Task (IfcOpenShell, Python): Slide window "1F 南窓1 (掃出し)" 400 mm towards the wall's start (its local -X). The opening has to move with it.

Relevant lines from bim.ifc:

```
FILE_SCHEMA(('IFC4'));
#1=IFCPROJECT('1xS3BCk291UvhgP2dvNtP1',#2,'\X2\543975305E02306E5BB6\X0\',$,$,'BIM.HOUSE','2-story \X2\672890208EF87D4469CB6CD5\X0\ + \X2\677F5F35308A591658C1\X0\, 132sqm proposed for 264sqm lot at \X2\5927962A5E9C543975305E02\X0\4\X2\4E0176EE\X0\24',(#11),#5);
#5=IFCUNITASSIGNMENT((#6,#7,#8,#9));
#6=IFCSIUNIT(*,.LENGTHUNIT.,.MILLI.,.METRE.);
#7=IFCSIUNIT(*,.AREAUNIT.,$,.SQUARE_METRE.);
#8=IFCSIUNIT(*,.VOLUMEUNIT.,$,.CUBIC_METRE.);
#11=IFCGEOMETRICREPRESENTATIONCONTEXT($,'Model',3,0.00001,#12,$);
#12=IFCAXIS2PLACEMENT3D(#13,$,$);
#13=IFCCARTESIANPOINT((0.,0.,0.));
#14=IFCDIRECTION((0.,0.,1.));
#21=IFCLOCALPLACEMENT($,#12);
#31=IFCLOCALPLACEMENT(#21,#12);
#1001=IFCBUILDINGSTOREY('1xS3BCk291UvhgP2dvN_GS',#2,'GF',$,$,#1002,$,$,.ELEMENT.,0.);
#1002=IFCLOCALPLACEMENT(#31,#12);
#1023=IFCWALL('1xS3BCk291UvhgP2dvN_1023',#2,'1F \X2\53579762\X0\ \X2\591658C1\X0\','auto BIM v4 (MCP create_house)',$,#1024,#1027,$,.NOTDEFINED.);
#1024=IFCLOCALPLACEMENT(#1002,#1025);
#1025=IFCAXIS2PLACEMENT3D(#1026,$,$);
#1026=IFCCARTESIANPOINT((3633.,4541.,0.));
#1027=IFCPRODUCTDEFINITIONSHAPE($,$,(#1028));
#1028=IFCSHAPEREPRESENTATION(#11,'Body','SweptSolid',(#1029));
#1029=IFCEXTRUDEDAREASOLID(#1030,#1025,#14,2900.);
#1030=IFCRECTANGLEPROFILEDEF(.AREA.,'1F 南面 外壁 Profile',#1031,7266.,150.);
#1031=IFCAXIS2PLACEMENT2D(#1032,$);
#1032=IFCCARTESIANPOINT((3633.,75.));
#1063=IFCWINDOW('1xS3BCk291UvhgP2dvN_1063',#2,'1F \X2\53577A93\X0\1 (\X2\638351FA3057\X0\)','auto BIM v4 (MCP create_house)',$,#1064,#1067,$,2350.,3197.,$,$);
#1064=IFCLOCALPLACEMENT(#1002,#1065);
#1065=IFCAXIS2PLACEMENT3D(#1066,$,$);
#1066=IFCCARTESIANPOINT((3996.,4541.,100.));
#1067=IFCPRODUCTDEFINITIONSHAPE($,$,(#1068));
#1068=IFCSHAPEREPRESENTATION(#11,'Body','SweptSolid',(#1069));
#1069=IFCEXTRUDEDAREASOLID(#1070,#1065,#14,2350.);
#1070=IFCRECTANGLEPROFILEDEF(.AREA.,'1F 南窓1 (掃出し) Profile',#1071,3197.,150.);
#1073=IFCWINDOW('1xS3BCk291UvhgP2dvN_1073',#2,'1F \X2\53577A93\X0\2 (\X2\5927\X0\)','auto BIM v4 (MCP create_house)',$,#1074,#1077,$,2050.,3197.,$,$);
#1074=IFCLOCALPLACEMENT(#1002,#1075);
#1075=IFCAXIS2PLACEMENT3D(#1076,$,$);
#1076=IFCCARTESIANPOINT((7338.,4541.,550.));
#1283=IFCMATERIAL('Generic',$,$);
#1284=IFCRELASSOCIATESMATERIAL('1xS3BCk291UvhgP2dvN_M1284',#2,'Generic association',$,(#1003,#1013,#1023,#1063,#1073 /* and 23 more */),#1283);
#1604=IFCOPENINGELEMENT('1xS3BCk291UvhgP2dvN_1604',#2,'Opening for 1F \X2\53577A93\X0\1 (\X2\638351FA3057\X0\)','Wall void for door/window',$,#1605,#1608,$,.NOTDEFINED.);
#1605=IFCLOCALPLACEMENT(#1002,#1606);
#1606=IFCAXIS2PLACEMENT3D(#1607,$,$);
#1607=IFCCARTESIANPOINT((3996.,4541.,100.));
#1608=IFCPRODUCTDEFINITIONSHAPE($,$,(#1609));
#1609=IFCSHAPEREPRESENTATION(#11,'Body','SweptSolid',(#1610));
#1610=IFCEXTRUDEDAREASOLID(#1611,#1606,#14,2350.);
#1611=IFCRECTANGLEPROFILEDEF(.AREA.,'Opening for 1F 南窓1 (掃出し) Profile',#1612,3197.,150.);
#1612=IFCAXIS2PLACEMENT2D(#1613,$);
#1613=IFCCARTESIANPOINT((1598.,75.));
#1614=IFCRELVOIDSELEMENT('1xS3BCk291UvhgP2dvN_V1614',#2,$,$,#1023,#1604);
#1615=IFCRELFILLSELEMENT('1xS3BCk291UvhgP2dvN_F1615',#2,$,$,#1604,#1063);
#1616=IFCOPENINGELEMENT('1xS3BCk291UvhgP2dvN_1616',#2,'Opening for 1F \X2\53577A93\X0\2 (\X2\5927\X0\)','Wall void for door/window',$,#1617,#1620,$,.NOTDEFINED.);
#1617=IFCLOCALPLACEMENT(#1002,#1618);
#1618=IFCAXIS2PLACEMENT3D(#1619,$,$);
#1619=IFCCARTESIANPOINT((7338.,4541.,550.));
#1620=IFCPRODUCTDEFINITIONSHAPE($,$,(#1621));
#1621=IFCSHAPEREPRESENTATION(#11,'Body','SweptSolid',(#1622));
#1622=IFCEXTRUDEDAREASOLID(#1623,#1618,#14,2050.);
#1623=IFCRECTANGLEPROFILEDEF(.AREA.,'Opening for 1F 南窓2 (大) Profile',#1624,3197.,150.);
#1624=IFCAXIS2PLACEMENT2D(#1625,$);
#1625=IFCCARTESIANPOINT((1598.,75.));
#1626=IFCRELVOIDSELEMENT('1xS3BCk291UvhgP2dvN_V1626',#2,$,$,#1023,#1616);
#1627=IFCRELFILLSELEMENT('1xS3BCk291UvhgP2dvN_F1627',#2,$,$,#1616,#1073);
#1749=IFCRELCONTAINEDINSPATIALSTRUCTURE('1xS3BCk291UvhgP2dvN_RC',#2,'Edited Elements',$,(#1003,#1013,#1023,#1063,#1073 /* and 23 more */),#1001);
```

```python
import ifcopenshell
import ifcopenshell.api.geometry
import ifcopenshell.util.placement
import ifcopenshell.util.unit

model = ifcopenshell.open("bim.ifc")
unit_scale = ifcopenshell.util.unit.calculate_unit_scale(model)

window = model.by_guid("1xS3BCk291UvhgP2dvN_1063")
opening = window.FillsVoids[0].RelatingOpeningElement
wall = opening.VoidsElements[0].RelatingBuildingElement

wall_matrix = ifcopenshell.util.placement.get_local_placement(wall.ObjectPlacement)
shift = wall_matrix[:3, 0] * -0.4 / unit_scale
before = ifcopenshell.util.placement.get_local_placement(window.ObjectPlacement)[:3, 3].copy()

# The window is not placed relative to its opening, so move both.
for product in (opening, window):
    matrix = ifcopenshell.util.placement.get_local_placement(product.ObjectPlacement)
    matrix[:3, 3] += shift
    ifcopenshell.api.geometry.edit_object_placement(model, product=product, matrix=matrix, is_si=False)

after = ifcopenshell.util.placement.get_local_placement(window.ObjectPlacement)[:3, 3]
print("window moved by", (after - before).round(3) + 0.0)

model.write("bim_edited.ifc")
```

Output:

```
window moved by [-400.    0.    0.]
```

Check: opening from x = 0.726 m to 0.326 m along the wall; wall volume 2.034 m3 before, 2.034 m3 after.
